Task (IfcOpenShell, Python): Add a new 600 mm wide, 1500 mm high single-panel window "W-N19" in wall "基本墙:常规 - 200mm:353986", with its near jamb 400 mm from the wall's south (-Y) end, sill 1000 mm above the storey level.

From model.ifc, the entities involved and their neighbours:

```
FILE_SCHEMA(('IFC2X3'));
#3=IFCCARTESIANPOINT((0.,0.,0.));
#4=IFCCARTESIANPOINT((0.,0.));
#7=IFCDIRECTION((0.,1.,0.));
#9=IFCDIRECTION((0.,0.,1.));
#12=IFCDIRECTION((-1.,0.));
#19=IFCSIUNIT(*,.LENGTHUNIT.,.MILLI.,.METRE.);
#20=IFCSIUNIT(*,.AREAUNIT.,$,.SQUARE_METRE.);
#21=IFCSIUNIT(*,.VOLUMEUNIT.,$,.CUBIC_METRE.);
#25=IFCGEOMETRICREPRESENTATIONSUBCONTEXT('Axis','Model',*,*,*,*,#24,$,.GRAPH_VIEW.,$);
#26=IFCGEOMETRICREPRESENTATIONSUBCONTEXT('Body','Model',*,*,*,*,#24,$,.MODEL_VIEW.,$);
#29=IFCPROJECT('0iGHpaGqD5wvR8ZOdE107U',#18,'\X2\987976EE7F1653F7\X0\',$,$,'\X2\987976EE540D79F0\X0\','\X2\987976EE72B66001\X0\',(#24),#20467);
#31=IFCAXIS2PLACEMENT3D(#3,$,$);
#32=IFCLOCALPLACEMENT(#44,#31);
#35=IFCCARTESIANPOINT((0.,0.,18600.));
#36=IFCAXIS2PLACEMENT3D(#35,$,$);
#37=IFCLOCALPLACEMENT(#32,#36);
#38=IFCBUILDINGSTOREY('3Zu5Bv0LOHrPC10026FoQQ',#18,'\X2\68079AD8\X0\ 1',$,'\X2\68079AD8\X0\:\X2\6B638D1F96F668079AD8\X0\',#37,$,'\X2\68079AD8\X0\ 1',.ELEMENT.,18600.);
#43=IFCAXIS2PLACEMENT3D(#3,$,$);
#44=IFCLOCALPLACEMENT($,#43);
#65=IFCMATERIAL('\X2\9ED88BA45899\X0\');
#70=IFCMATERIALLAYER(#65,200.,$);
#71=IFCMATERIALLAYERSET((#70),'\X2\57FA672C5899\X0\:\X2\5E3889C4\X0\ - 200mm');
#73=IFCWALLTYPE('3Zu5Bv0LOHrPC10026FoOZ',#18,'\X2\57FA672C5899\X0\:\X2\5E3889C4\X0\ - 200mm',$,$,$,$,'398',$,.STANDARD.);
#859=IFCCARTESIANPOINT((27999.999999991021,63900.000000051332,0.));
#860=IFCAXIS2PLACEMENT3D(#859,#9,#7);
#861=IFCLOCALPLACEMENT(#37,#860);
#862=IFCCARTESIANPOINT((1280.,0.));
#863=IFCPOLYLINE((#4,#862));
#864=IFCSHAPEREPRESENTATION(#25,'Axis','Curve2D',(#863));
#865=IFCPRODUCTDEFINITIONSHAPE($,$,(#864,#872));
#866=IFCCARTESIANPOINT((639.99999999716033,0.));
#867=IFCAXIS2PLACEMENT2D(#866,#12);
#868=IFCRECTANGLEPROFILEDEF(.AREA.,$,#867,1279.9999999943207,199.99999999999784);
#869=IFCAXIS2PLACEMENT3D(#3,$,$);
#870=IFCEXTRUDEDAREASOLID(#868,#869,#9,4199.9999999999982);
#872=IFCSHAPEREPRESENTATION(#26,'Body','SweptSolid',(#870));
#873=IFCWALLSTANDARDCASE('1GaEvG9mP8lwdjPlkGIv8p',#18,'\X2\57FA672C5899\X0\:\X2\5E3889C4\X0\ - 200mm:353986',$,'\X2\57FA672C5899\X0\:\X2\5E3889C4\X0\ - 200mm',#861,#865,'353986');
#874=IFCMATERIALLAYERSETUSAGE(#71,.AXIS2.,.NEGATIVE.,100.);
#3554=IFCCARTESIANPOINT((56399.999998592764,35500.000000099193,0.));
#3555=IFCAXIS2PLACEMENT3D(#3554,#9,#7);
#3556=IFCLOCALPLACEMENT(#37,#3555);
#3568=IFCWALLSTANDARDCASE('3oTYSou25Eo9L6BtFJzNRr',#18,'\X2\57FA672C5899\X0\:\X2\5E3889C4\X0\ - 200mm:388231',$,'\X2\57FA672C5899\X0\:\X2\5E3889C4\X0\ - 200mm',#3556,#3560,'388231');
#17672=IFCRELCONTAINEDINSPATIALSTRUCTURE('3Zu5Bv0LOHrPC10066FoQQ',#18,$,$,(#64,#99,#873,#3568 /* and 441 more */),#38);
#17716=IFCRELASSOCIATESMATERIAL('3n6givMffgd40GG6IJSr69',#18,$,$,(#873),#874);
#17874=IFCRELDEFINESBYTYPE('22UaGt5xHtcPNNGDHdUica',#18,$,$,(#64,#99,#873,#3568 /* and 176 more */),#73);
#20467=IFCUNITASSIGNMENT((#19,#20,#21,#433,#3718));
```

```python
import numpy as np
import ifcopenshell
import ifcopenshell.api.feature
import ifcopenshell.api.geometry
import ifcopenshell.api.root
import ifcopenshell.api.spatial
import ifcopenshell.api.type
import ifcopenshell.geom
import ifcopenshell.util.element
import ifcopenshell.util.placement
import ifcopenshell.util.representation
import ifcopenshell.util.shape
import ifcopenshell.util.unit

model = ifcopenshell.open("model.ifc")
unit_scale = ifcopenshell.util.unit.calculate_unit_scale(model)
settings = ifcopenshell.geom.settings()


def volume(element):
    """Net volume in cubic metres, openings subtracted."""
    shape = ifcopenshell.geom.create_shape(settings, element)
    return ifcopenshell.util.shape.get_volume(shape.geometry)


wall = model.by_guid("1GaEvG9mP8lwdjPlkGIv8p")
storey = ifcopenshell.util.element.get_container(wall, ifc_class="IfcBuildingStorey")
context = ifcopenshell.util.representation.get_context(model, "Model", "Body", "MODEL_VIEW")
before = volume(wall)

width, height, from_end, sill = 0.6, 1.5, 0.4, 1  # metres

# The wall runs along its own X axis, and the end named is its -X end.
wall_shape = ifcopenshell.geom.create_shape(settings, wall)
x, y, z = ifcopenshell.util.shape.get_vertices(wall_shape.geometry).T
start = x.min() + from_end
face, thickness = float(y.min()), float(y.max() - y.min())
wall_matrix = ifcopenshell.util.placement.get_local_placement(wall.ObjectPlacement)
level = ifcopenshell.util.placement.get_local_placement(storey.ObjectPlacement)[2, 3]


def in_wall(x, y):
    """Placement at x, y metres in the wall's axes, at sill height."""
    matrix = wall_matrix.copy()
    matrix[:, 3] = wall_matrix @ np.array([x / unit_scale, y / unit_scale, 0.0, 1.0])
    matrix[2, 3] = level + sill / unit_scale
    return matrix


# Opening: a box that overshoots both wall faces by 50 mm.
opening = ifcopenshell.api.root.create_entity(model, ifc_class="IfcOpeningElement")
box = ifcopenshell.api.geometry.add_wall_representation(
    model, context=context, length=width, height=height, thickness=thickness + 0.1
)
ifcopenshell.api.geometry.assign_representation(model, product=opening, representation=box)
ifcopenshell.api.geometry.edit_object_placement(model, product=opening, matrix=in_wall(start, face - 0.05), is_si=False)
ifcopenshell.api.feature.add_feature(model, feature=opening, element=wall)

window = ifcopenshell.api.root.create_entity(model, ifc_class="IfcWindow", name="W-N19")
window.OverallWidth, window.OverallHeight = width / unit_scale, height / unit_scale
body = ifcopenshell.api.geometry.add_window_representation(
    model,
    context=context,
    overall_width=window.OverallWidth,
    overall_height=window.OverallHeight,
    partition_type="SINGLE_PANEL",
)
ifcopenshell.api.geometry.assign_representation(model, product=window, representation=body)
ifcopenshell.api.spatial.assign_container(model, products=[window], relating_structure=storey)
fills = ifcopenshell.api.feature.add_filling(model, opening=opening, element=window)
fills.OwnerHistory = window.OwnerHistory  # required in IFC2X3

# IFC2X3 keeps the operation on the window style.
style = ifcopenshell.api.root.create_entity(model, ifc_class="IfcWindowStyle", name="W-N19")
style.OperationType, style.ConstructionType = "SINGLE_PANEL", "NOTDEFINED"
style.ParameterTakesPrecedence = style.Sizeable = False
ifcopenshell.api.type.assign_type(model, related_objects=[window], relating_type=style)

# Centre the window in the wall's thickness.
ifcopenshell.api.geometry.edit_object_placement(model, product=window, matrix=in_wall(start, face), is_si=False)
window_shape = ifcopenshell.geom.create_shape(settings, window)
depth = ifcopenshell.util.shape.get_vertices(window_shape.geometry)[:, 1]
offset = face + thickness / 2 - (depth.min() + depth.max()) / 2
ifcopenshell.api.geometry.edit_object_placement(model, product=window, matrix=in_wall(start, offset), is_si=False)

after = volume(wall)

print(f"wall volume {before:.3f} -> {after:.3f} m3")

model.write("model_rev.ifc")
```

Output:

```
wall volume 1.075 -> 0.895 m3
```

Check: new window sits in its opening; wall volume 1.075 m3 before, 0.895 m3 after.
